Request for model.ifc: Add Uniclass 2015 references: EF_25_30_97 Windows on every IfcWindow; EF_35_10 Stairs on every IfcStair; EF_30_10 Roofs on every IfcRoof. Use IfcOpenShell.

First a look at what the model holds.

```python
import ifcopenshell

model = ifcopenshell.open("model.ifc")
print(model.schema)
print("classifications:", [c.Name for c in model.by_type("IfcClassification")])
for ifc_class in ("IfcDoor", "IfcRoof", "IfcStair", "IfcWall", "IfcWindow"):
    print(ifc_class, len(model.by_type(ifc_class)))
```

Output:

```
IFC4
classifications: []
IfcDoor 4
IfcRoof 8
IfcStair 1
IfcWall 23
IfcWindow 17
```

```python
import ifcopenshell
import ifcopenshell.api.classification

model = ifcopenshell.open("model.ifc")

system = ifcopenshell.api.classification.add_classification(model, classification="Uniclass 2015")

codes = {
    "IfcWindow": ("EF_25_30_97", "Windows"),
    "IfcStair": ("EF_35_10", "Stairs"),
    "IfcRoof": ("EF_30_10", "Roofs"),
}
for ifc_class, (code, name) in codes.items():
    products = model.by_type(ifc_class)
    ifcopenshell.api.classification.add_reference(
        model, products=products, classification=system, identification=code, name=name
    )
    print(code, len(products))

model.write("model_edited.ifc")
```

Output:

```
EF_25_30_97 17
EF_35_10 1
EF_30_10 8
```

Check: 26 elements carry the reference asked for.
